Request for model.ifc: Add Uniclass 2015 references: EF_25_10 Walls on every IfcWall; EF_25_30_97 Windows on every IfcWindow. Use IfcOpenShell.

First a look at what the model holds.

```python
import ifcopenshell

model = ifcopenshell.open("model.ifc")
print(model.schema)
print("classifications:", [c.Name for c in model.by_type("IfcClassification")])
for ifc_class in ("IfcDoor", "IfcRoof", "IfcStair", "IfcWall", "IfcWindow"):
    print(ifc_class, len(model.by_type(ifc_class)))
```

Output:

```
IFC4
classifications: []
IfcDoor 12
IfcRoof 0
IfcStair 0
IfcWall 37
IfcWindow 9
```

```python
import ifcopenshell
import ifcopenshell.api.classification

model = ifcopenshell.open("model.ifc")

system = ifcopenshell.api.classification.add_classification(model, classification="Uniclass 2015")

codes = {
    "IfcWall": ("EF_25_10", "Walls"),
    "IfcWindow": ("EF_25_30_97", "Windows"),
}
for ifc_class, (code, name) in codes.items():
    products = model.by_type(ifc_class)
    ifcopenshell.api.classification.add_reference(
        model, products=products, classification=system, identification=code, name=name
    )
    print(code, len(products))

model.write("model_v2.ifc")
```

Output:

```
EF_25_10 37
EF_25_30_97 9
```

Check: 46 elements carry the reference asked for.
